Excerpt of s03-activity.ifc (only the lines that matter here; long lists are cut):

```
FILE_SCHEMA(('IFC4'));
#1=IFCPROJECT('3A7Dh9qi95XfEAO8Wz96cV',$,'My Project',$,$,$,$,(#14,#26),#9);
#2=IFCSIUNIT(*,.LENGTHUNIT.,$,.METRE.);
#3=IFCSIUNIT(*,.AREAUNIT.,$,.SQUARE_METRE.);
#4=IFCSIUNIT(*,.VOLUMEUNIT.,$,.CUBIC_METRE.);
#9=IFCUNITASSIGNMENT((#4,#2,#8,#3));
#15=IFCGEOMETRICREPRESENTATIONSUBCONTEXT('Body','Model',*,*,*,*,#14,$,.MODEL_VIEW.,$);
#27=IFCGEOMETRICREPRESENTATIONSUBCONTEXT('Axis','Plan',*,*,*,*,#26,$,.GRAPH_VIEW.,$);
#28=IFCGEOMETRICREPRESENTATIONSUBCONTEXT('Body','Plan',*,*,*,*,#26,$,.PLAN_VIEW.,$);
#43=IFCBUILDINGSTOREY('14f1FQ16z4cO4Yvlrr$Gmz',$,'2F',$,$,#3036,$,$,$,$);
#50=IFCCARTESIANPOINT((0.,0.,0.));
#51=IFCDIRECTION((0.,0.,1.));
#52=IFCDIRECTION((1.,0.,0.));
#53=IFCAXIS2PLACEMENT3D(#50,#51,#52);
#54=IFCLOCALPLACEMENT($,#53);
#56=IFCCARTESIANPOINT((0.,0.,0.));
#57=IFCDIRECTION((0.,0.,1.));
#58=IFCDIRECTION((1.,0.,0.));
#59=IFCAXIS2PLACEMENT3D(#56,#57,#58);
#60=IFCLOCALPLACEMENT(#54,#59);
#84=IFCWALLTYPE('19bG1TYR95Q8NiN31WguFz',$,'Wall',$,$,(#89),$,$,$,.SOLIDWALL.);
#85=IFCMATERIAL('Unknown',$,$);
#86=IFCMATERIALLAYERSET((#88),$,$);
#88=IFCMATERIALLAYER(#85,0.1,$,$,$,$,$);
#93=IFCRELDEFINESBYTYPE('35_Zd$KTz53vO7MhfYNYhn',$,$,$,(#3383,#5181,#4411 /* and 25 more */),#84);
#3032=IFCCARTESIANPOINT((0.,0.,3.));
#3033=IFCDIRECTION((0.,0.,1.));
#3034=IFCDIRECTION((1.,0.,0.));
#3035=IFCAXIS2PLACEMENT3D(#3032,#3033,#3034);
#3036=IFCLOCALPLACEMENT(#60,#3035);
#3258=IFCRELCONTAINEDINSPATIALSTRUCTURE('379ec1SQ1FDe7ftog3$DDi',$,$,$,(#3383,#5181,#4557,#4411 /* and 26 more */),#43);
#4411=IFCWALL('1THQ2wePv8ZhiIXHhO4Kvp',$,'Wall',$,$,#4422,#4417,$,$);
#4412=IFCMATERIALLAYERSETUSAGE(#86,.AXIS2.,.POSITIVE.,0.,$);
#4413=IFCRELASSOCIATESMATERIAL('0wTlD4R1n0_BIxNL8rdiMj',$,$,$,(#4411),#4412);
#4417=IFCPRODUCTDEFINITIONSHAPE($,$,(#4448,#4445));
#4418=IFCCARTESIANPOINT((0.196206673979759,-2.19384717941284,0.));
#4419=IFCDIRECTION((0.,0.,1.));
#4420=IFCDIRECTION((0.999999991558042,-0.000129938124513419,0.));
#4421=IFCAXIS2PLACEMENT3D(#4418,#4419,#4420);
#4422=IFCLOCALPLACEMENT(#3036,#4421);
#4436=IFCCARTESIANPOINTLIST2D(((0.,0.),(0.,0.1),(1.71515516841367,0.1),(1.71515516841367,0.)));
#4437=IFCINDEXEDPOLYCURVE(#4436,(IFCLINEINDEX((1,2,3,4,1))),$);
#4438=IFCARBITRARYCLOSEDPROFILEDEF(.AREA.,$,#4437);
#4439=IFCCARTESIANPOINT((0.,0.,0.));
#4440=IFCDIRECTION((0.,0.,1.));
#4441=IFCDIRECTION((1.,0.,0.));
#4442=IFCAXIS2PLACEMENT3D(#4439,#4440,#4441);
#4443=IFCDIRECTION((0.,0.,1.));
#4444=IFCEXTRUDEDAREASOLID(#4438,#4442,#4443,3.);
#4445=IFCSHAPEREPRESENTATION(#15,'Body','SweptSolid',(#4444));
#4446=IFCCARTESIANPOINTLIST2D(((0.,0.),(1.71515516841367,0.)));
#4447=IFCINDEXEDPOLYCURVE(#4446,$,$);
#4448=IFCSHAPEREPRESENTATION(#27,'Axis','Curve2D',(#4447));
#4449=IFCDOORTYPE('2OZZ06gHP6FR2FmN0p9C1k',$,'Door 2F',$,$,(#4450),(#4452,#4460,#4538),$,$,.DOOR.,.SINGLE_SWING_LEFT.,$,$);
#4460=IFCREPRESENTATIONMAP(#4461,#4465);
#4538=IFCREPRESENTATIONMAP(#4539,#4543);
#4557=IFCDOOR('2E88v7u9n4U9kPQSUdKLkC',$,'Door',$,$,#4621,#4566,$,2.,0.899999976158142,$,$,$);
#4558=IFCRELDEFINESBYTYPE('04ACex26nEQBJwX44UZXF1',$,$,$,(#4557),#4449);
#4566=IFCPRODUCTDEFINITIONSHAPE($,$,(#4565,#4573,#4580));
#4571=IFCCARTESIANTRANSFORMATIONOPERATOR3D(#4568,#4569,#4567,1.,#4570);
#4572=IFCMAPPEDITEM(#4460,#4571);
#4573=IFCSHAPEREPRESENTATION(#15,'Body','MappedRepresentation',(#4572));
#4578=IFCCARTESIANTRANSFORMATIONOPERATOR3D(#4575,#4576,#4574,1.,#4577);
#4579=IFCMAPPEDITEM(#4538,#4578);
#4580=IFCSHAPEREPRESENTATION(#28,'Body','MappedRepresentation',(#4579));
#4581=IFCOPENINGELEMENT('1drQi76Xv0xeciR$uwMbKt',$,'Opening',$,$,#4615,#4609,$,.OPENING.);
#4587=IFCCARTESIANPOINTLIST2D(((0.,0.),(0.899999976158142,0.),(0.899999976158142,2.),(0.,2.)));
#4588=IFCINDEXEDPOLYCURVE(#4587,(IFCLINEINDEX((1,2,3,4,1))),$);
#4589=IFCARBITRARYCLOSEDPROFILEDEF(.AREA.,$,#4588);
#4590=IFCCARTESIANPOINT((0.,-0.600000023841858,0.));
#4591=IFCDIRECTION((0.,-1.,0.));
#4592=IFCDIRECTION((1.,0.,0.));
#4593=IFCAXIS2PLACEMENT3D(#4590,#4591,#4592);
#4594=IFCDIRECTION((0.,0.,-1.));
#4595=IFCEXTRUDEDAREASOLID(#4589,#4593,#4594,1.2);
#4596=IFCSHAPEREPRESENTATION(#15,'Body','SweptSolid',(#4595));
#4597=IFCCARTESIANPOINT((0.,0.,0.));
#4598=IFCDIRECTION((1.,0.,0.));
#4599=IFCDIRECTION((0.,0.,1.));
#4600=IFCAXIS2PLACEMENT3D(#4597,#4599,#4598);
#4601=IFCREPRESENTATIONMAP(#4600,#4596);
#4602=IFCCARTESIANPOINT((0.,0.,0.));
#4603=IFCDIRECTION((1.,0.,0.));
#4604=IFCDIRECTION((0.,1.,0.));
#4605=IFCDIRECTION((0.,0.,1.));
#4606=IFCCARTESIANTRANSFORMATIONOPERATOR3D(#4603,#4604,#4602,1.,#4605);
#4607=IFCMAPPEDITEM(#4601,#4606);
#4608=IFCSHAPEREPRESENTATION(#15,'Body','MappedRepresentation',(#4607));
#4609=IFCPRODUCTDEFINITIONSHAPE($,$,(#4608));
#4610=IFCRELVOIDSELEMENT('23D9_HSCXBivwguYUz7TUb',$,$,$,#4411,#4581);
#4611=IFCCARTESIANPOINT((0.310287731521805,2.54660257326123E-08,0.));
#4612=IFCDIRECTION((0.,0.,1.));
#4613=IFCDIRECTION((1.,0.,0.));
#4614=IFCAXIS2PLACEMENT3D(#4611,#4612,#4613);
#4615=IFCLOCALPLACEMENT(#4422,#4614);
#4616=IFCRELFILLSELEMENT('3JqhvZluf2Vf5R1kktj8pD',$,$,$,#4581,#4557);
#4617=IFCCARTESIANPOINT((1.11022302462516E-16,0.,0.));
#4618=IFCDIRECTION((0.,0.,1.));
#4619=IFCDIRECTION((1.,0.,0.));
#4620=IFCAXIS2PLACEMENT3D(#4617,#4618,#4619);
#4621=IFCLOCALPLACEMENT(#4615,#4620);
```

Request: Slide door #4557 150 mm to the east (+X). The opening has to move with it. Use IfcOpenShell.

```python
import ifcopenshell
import ifcopenshell.api.geometry
import ifcopenshell.util.placement
import ifcopenshell.util.unit

model = ifcopenshell.open("s03-activity.ifc")
unit_scale = ifcopenshell.util.unit.calculate_unit_scale(model)

door = model.by_id(4557)
opening = door.FillsVoids[0].RelatingOpeningElement
wall = opening.VoidsElements[0].RelatingBuildingElement

wall_matrix = ifcopenshell.util.placement.get_local_placement(wall.ObjectPlacement)
shift = wall_matrix[:3, 0] * 0.15 / unit_scale
before = ifcopenshell.util.placement.get_local_placement(door.ObjectPlacement)[:3, 3].copy()

# The door is placed relative to its opening, so it follows when the opening moves.
matrix = ifcopenshell.util.placement.get_local_placement(opening.ObjectPlacement)
matrix[:3, 3] += shift
ifcopenshell.api.geometry.edit_object_placement(
    model, product=opening, matrix=matrix, is_si=False, should_transform_children=True
)

after = ifcopenshell.util.placement.get_local_placement(door.ObjectPlacement)[:3, 3]
print("door moved by", (after - before).round(3) + 0.0)

model.write("s03-activity_edited.ifc")
```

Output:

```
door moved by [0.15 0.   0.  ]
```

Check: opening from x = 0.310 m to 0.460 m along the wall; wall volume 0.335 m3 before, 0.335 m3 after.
